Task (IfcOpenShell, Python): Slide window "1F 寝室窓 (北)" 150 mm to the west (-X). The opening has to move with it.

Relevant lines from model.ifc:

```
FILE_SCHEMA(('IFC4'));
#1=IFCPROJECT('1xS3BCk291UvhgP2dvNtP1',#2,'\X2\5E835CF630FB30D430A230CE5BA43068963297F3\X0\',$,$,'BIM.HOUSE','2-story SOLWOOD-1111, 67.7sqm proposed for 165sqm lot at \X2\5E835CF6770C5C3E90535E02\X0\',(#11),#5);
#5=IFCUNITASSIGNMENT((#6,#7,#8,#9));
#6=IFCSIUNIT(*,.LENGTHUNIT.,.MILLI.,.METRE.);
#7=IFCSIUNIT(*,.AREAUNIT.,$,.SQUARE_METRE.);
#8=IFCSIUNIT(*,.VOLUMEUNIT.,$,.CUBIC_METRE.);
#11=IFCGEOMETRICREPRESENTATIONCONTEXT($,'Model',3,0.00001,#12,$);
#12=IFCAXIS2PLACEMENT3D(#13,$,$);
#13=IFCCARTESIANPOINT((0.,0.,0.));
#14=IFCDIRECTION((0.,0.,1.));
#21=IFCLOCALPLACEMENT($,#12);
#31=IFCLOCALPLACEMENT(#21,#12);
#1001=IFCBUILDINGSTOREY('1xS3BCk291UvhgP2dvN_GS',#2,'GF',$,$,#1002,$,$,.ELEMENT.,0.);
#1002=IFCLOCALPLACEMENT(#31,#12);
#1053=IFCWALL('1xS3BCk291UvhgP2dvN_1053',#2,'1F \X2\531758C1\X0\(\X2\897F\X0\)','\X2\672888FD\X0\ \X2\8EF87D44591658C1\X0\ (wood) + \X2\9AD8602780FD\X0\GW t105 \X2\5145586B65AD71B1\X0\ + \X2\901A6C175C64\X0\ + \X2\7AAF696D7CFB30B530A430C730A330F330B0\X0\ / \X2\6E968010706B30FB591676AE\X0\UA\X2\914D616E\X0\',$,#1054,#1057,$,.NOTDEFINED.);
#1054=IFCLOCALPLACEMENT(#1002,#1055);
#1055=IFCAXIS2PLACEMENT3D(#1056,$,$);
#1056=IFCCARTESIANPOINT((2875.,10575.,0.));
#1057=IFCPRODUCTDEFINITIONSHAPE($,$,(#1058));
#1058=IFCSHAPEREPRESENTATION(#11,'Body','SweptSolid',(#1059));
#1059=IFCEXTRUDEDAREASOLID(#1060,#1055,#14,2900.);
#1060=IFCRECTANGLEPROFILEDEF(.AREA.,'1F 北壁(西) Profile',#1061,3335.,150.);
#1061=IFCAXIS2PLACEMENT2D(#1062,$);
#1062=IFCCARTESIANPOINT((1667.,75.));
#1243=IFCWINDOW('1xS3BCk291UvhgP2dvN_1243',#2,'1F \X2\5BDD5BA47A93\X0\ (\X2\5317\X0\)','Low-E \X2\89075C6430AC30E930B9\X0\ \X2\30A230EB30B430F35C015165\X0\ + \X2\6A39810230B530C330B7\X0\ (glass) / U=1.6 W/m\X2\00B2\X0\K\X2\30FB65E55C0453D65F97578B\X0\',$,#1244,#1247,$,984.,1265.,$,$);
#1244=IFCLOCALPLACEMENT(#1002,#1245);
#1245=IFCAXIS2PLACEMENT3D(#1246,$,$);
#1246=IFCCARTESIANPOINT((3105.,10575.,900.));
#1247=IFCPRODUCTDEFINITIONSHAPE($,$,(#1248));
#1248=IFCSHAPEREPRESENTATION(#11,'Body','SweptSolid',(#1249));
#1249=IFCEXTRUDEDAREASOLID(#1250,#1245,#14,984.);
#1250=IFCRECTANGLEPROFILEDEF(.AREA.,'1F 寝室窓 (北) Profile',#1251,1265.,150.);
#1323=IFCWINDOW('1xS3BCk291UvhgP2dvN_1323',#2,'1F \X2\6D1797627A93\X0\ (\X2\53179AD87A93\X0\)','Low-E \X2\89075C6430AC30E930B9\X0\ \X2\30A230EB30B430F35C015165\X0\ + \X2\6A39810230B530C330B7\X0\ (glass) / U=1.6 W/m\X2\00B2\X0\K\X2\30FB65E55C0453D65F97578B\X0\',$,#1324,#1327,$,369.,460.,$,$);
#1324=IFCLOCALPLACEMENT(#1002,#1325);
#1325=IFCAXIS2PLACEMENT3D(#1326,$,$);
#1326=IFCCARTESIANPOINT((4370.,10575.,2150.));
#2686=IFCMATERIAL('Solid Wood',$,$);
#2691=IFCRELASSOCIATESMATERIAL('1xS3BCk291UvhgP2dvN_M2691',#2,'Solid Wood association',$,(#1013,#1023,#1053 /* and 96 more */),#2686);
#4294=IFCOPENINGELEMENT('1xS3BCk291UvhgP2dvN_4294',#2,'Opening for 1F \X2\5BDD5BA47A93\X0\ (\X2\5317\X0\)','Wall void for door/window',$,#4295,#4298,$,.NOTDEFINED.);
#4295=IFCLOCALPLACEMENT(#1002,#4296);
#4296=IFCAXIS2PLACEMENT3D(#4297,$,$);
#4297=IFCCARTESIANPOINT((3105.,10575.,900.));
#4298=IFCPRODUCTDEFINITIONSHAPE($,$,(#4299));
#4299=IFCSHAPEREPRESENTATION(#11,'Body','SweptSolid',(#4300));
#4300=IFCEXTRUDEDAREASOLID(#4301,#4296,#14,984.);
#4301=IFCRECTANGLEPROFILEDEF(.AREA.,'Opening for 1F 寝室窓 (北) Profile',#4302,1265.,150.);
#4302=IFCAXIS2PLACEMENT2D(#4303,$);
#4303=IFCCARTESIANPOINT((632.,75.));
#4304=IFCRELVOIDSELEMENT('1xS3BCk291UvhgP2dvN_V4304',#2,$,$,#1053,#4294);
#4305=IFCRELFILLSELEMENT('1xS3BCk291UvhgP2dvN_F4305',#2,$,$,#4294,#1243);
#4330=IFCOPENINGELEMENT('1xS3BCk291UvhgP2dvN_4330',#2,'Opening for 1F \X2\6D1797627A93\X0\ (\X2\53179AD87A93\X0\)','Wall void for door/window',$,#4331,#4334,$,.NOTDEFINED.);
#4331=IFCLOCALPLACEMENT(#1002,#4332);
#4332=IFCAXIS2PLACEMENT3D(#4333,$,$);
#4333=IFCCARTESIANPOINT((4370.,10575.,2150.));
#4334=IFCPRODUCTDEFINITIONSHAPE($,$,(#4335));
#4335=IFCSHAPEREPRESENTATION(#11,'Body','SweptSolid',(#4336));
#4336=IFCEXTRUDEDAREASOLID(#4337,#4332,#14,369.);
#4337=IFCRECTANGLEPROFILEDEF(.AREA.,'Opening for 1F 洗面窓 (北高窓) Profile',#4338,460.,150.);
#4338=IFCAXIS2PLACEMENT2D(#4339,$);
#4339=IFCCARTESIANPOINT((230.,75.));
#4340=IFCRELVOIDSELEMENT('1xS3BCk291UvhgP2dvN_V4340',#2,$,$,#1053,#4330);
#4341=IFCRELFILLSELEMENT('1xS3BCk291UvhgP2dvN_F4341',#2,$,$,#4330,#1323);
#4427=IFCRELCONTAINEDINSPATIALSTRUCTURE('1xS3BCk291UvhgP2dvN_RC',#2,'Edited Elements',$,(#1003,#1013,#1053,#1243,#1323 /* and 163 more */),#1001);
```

```python
import ifcopenshell
import ifcopenshell.api.geometry
import ifcopenshell.util.placement
import ifcopenshell.util.unit

model = ifcopenshell.open("model.ifc")
unit_scale = ifcopenshell.util.unit.calculate_unit_scale(model)

window = model.by_guid("1xS3BCk291UvhgP2dvN_1243")
opening = window.FillsVoids[0].RelatingOpeningElement
wall = opening.VoidsElements[0].RelatingBuildingElement

wall_matrix = ifcopenshell.util.placement.get_local_placement(wall.ObjectPlacement)
shift = wall_matrix[:3, 0] * -0.15 / unit_scale
before = ifcopenshell.util.placement.get_local_placement(window.ObjectPlacement)[:3, 3].copy()

# The window is not placed relative to its opening, so move both.
for product in (opening, window):
    matrix = ifcopenshell.util.placement.get_local_placement(product.ObjectPlacement)
    matrix[:3, 3] += shift
    ifcopenshell.api.geometry.edit_object_placement(model, product=product, matrix=matrix, is_si=False)

after = ifcopenshell.util.placement.get_local_placement(window.ObjectPlacement)[:3, 3]
print("window moved by", (after - before).round(3) + 0.0)

model.write("model_rev.ifc")
```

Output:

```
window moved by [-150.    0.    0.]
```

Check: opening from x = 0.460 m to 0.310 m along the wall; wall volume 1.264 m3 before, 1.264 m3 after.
